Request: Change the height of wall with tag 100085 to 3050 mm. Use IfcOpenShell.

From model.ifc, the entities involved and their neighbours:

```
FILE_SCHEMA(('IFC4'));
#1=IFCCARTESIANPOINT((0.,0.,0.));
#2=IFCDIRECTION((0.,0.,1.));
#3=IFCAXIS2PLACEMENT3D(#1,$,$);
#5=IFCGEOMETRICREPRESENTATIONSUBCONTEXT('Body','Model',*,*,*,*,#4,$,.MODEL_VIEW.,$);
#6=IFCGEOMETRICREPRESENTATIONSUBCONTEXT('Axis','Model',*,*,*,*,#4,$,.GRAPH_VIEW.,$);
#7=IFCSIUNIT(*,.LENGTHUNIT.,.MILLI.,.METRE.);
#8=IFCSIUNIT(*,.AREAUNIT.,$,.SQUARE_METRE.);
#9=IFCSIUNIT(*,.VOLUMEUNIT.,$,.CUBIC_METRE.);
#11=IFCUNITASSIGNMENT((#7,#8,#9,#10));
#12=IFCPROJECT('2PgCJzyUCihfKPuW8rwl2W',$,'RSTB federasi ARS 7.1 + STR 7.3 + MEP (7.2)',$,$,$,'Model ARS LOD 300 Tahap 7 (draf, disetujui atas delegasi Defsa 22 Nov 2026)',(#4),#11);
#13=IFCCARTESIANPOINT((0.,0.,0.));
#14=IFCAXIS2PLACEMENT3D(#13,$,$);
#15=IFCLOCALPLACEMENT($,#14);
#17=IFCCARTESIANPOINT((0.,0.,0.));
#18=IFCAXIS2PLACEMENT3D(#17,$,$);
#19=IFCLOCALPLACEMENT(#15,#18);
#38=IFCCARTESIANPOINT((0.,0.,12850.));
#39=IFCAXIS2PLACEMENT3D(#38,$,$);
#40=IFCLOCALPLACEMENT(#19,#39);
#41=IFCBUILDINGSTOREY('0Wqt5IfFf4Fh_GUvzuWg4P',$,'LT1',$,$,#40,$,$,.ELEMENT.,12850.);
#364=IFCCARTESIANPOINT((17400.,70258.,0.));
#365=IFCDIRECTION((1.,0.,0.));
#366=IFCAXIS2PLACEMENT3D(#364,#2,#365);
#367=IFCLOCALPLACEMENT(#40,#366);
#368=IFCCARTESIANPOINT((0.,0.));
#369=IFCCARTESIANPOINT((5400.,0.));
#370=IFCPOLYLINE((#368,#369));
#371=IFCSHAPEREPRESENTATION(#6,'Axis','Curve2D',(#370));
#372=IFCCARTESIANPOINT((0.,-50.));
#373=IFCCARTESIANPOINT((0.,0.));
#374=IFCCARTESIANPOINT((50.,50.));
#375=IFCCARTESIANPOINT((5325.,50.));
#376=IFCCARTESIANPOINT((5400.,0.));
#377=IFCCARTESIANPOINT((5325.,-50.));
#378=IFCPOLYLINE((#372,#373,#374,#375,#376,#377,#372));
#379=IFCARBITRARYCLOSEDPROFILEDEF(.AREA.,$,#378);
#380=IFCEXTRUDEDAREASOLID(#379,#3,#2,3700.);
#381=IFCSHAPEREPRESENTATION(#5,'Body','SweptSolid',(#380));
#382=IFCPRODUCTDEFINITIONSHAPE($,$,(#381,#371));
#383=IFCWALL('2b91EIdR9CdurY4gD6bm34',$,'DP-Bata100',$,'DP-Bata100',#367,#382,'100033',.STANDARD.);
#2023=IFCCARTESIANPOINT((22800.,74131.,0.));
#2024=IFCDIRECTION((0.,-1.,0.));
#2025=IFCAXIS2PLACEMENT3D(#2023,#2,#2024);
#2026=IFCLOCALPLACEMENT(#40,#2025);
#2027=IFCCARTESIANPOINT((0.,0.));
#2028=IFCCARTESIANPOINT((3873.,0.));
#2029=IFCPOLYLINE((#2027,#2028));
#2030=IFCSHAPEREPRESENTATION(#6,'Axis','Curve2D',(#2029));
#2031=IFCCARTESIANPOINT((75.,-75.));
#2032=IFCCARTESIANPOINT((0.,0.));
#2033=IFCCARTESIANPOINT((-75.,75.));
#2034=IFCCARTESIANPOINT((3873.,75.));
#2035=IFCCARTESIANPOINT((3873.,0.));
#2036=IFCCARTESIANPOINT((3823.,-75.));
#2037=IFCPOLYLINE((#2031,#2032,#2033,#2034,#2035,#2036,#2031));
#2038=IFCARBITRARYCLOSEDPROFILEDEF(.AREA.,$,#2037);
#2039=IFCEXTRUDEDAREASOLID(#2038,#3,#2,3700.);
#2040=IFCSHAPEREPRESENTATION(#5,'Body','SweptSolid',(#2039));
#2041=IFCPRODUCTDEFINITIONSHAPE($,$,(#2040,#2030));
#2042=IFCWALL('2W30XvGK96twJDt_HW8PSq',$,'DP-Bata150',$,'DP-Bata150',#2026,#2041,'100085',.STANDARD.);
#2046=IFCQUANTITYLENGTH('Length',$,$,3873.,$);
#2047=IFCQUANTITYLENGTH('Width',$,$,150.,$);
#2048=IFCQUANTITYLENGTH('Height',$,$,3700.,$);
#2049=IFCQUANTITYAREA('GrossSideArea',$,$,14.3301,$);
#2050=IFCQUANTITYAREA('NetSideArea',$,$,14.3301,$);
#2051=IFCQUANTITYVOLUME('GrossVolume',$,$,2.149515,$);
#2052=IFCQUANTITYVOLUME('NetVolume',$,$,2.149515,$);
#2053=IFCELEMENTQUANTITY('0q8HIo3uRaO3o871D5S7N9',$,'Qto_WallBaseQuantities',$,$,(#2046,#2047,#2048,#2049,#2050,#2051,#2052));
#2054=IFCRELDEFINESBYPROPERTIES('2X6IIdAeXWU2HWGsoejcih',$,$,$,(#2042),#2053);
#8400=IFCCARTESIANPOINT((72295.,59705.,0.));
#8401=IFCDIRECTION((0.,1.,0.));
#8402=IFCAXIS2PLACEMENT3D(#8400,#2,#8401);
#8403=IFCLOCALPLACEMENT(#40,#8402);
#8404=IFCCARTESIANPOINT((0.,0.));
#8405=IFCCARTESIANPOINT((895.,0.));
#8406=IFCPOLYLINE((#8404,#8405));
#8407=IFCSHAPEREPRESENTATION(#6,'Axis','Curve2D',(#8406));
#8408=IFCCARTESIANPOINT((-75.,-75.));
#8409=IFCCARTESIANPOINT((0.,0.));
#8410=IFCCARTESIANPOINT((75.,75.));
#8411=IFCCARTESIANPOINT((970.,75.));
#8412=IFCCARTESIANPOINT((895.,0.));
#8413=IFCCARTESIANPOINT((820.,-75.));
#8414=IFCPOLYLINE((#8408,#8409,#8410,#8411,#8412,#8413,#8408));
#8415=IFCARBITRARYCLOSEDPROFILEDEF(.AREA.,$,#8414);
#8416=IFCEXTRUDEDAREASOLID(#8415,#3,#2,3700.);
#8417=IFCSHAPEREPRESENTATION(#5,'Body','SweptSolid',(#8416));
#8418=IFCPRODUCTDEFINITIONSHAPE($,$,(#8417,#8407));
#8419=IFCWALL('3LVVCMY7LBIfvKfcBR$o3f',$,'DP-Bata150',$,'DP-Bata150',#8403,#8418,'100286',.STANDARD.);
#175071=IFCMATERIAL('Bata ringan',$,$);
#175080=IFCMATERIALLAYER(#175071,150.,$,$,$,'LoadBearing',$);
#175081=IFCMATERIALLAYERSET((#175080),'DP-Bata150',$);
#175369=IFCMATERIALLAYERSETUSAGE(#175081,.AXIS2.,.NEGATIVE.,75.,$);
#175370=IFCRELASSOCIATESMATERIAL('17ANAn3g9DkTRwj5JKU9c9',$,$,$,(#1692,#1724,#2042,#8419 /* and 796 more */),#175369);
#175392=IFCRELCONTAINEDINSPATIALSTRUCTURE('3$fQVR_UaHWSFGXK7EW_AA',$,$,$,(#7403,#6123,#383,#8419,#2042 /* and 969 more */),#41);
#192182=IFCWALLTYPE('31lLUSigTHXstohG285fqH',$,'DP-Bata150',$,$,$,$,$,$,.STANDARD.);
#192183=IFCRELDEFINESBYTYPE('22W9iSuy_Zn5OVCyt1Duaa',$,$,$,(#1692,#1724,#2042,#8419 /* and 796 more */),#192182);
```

```python
import ifcopenshell
import ifcopenshell.api.pset
import ifcopenshell.geom
import ifcopenshell.util.element
import ifcopenshell.util.representation
import ifcopenshell.util.shape
import ifcopenshell.util.unit

model = ifcopenshell.open("model.ifc")
unit_scale = ifcopenshell.util.unit.calculate_unit_scale(model)
area_scale = ifcopenshell.util.unit.calculate_unit_scale(model, "AREAUNIT")
volume_scale = ifcopenshell.util.unit.calculate_unit_scale(model, "VOLUMEUNIT")
settings = ifcopenshell.geom.settings()


def volume(element):
    """Net volume in cubic metres, openings subtracted."""
    shape = ifcopenshell.geom.create_shape(settings, element)
    return ifcopenshell.util.shape.get_volume(shape.geometry)


wall = model.by_guid("2W30XvGK96twJDt_HW8PSq")
before = volume(wall)

body = ifcopenshell.util.representation.get_representation(wall, "Model", "Body")
solid = body.Items[0]
old_height = solid.Depth
solid.Depth = 3050.0
after = volume(wall)
thickness = 0.15  # wall thickness in metres

# Update the stored height, areas and volumes.
qto = model.by_id(ifcopenshell.util.element.get_pset(wall, "Qto_WallBaseQuantities", should_inherit=False)["id"])
ifcopenshell.api.pset.edit_qto(model, qto=qto, properties={
    "Height": solid.Depth,
    "GrossSideArea": ifcopenshell.util.element.get_pset(wall, "Qto_WallBaseQuantities", "GrossSideArea") * solid.Depth / old_height,
    "NetSideArea": after / thickness / area_scale,
    "GrossVolume": ifcopenshell.util.element.get_pset(wall, "Qto_WallBaseQuantities", "GrossVolume") * solid.Depth / old_height,
    "NetVolume": after / volume_scale,
})

print(f"height {old_height:g} -> {solid.Depth:g}, volume {before:.3f} -> {after:.3f} m3")

model.write("model_rev.ifc")
```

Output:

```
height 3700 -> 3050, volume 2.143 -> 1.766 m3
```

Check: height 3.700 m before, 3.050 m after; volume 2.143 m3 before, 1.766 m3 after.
